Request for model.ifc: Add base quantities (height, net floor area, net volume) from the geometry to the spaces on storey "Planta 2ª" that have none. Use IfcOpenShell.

First a look at what the model holds.

```python
import ifcopenshell
import ifcopenshell.util.element
import ifcopenshell.util.unit

model = ifcopenshell.open("model.ifc")
print(model.schema)
for unit_type in ("LENGTHUNIT", "AREAUNIT", "VOLUMEUNIT"):
    print(unit_type, ifcopenshell.util.unit.calculate_unit_scale(model, unit_type))
storey = next(s for s in model.by_type("IfcBuildingStorey") if s.Name == "Planta 2ª")
spaces = [e for e in ifcopenshell.util.element.get_decomposition(storey) if e.is_a("IfcSpace")]
for e in sorted(spaces, key=lambda e: e.id()):
    print(e.id(), e.is_a(), e.Name, list(ifcopenshell.util.element.get_psets(e, qtos_only=True)), sep=" | ")
```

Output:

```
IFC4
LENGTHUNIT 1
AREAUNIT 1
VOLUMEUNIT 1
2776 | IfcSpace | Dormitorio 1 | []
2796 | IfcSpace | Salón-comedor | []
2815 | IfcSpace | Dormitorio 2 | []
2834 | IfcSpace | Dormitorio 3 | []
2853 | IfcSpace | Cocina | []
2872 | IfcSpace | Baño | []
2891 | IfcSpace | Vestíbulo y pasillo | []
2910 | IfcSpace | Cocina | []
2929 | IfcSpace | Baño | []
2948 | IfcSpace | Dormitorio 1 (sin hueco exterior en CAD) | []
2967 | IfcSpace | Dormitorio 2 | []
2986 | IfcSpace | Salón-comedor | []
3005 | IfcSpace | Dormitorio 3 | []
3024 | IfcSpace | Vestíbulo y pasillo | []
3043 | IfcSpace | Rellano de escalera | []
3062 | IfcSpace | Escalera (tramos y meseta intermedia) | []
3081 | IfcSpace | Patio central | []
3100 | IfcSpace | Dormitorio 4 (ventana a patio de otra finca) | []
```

```python
import ifcopenshell
import ifcopenshell.api.pset
import ifcopenshell.geom
import ifcopenshell.util.element
import ifcopenshell.util.shape
import ifcopenshell.util.unit

model = ifcopenshell.open("model.ifc")
unit_scale = ifcopenshell.util.unit.calculate_unit_scale(model)
area_scale = ifcopenshell.util.unit.calculate_unit_scale(model, "AREAUNIT")
volume_scale = ifcopenshell.util.unit.calculate_unit_scale(model, "VOLUMEUNIT")
settings = ifcopenshell.geom.settings()

storey = next(s for s in model.by_type("IfcBuildingStorey") if s.Name == "Planta 2ª")
spaces = [e for e in ifcopenshell.util.element.get_decomposition(storey) if e.is_a("IfcSpace")]

for e in sorted(spaces, key=lambda e: e.id()):
    if ifcopenshell.util.element.get_psets(e, qtos_only=True, should_inherit=False):
        continue
    # Geometry comes back in metres, in the element's own axes.
    shape = ifcopenshell.geom.create_shape(settings, e)
    values = {
        "Height": ifcopenshell.util.shape.get_z(shape.geometry) / unit_scale,
        "NetFloorArea": ifcopenshell.util.shape.get_footprint_area(shape.geometry) / area_scale,
        "NetVolume": ifcopenshell.util.shape.get_volume(shape.geometry) / volume_scale,
    }
    qto = ifcopenshell.api.pset.add_qto(model, product=e, name="Qto_SpaceBaseQuantities")
    ifcopenshell.api.pset.edit_qto(model, qto=qto, properties=values)
    print(e.id(), {k: round(v, 3) for k, v in values.items()})

model.write("model_edited.ifc")
```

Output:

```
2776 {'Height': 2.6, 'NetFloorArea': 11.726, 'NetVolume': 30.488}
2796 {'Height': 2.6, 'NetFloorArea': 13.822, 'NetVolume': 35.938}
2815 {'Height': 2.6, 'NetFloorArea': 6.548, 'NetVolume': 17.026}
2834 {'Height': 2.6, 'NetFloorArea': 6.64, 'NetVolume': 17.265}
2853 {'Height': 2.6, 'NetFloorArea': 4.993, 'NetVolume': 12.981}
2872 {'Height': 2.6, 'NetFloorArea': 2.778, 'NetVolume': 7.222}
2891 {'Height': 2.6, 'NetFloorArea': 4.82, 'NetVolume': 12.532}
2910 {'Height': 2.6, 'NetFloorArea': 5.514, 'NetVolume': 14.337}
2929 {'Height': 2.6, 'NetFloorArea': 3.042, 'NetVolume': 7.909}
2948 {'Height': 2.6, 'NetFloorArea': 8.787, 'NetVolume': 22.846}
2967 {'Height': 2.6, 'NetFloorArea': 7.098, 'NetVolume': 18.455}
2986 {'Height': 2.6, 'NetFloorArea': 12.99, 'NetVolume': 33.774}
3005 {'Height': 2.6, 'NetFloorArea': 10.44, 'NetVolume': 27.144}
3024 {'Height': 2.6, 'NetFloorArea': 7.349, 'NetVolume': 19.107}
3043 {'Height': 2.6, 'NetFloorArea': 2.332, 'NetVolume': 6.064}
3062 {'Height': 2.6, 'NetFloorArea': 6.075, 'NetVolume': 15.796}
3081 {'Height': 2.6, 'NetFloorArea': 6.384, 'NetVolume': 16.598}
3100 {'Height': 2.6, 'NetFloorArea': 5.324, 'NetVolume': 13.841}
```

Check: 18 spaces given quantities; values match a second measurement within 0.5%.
